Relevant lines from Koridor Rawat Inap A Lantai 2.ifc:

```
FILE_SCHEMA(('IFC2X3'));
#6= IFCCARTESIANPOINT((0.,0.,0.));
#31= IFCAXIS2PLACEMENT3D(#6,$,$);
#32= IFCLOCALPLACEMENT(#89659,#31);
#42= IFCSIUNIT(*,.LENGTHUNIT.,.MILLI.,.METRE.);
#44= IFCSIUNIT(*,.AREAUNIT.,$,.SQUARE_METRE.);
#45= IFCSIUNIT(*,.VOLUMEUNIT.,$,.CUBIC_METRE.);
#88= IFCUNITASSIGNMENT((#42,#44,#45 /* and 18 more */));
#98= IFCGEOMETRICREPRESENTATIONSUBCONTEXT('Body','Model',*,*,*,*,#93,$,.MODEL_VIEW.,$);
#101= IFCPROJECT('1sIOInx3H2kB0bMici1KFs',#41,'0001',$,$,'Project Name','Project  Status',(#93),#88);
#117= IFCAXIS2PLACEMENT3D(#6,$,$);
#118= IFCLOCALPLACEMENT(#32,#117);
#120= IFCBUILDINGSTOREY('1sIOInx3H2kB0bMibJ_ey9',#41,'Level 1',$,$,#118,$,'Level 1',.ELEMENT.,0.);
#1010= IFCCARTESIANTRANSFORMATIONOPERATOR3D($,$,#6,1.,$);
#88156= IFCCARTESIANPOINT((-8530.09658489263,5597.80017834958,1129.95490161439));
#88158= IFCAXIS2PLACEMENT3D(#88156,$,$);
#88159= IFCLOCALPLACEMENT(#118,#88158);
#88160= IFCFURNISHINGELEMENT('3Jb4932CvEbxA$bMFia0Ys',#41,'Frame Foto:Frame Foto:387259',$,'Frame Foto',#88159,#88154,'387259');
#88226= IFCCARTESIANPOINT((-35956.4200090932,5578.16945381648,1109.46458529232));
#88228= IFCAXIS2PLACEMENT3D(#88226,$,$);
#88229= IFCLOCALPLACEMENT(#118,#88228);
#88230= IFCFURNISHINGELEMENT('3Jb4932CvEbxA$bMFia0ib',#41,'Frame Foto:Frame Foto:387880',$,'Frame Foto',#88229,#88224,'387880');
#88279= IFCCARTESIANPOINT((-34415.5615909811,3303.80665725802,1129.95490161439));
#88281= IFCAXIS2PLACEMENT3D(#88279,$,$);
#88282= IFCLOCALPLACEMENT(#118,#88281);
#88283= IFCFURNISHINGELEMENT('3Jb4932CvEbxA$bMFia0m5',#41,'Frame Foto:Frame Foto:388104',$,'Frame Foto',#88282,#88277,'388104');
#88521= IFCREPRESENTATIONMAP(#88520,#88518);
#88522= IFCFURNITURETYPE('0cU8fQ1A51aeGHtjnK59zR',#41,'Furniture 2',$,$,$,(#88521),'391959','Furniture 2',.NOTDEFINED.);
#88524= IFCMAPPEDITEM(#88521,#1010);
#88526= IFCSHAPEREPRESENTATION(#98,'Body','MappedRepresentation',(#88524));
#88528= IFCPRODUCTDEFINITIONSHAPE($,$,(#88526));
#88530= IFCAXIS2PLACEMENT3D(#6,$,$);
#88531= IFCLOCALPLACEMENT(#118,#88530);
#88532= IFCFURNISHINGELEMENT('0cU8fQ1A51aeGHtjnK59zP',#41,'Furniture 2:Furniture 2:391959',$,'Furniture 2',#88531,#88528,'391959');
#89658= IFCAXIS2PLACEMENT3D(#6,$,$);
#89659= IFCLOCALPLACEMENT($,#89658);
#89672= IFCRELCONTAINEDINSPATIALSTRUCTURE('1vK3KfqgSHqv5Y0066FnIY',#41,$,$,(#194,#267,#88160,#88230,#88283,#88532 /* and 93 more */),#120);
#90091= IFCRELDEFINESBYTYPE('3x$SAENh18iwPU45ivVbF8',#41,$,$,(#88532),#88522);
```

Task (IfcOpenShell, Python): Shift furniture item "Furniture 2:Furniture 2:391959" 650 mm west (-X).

```python
import ifcopenshell
import ifcopenshell.api.geometry
import ifcopenshell.util.placement
import ifcopenshell.util.unit

model = ifcopenshell.open("Koridor Rawat Inap A Lantai 2.ifc")
unit_scale = ifcopenshell.util.unit.calculate_unit_scale(model)

item = model.by_id(88532)
matrix = ifcopenshell.util.placement.get_local_placement(item.ObjectPlacement)
matrix[0, 3] -= 0.65 / unit_scale
ifcopenshell.api.geometry.edit_object_placement(model, product=item, matrix=matrix, is_si=False)

print(ifcopenshell.util.placement.get_local_placement(item.ObjectPlacement).round(3) + 0.0)

model.write("Koridor Rawat Inap A Lantai 2-out.ifc")
```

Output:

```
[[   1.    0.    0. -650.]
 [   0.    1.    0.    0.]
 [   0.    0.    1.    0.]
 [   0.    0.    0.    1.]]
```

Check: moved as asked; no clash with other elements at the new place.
